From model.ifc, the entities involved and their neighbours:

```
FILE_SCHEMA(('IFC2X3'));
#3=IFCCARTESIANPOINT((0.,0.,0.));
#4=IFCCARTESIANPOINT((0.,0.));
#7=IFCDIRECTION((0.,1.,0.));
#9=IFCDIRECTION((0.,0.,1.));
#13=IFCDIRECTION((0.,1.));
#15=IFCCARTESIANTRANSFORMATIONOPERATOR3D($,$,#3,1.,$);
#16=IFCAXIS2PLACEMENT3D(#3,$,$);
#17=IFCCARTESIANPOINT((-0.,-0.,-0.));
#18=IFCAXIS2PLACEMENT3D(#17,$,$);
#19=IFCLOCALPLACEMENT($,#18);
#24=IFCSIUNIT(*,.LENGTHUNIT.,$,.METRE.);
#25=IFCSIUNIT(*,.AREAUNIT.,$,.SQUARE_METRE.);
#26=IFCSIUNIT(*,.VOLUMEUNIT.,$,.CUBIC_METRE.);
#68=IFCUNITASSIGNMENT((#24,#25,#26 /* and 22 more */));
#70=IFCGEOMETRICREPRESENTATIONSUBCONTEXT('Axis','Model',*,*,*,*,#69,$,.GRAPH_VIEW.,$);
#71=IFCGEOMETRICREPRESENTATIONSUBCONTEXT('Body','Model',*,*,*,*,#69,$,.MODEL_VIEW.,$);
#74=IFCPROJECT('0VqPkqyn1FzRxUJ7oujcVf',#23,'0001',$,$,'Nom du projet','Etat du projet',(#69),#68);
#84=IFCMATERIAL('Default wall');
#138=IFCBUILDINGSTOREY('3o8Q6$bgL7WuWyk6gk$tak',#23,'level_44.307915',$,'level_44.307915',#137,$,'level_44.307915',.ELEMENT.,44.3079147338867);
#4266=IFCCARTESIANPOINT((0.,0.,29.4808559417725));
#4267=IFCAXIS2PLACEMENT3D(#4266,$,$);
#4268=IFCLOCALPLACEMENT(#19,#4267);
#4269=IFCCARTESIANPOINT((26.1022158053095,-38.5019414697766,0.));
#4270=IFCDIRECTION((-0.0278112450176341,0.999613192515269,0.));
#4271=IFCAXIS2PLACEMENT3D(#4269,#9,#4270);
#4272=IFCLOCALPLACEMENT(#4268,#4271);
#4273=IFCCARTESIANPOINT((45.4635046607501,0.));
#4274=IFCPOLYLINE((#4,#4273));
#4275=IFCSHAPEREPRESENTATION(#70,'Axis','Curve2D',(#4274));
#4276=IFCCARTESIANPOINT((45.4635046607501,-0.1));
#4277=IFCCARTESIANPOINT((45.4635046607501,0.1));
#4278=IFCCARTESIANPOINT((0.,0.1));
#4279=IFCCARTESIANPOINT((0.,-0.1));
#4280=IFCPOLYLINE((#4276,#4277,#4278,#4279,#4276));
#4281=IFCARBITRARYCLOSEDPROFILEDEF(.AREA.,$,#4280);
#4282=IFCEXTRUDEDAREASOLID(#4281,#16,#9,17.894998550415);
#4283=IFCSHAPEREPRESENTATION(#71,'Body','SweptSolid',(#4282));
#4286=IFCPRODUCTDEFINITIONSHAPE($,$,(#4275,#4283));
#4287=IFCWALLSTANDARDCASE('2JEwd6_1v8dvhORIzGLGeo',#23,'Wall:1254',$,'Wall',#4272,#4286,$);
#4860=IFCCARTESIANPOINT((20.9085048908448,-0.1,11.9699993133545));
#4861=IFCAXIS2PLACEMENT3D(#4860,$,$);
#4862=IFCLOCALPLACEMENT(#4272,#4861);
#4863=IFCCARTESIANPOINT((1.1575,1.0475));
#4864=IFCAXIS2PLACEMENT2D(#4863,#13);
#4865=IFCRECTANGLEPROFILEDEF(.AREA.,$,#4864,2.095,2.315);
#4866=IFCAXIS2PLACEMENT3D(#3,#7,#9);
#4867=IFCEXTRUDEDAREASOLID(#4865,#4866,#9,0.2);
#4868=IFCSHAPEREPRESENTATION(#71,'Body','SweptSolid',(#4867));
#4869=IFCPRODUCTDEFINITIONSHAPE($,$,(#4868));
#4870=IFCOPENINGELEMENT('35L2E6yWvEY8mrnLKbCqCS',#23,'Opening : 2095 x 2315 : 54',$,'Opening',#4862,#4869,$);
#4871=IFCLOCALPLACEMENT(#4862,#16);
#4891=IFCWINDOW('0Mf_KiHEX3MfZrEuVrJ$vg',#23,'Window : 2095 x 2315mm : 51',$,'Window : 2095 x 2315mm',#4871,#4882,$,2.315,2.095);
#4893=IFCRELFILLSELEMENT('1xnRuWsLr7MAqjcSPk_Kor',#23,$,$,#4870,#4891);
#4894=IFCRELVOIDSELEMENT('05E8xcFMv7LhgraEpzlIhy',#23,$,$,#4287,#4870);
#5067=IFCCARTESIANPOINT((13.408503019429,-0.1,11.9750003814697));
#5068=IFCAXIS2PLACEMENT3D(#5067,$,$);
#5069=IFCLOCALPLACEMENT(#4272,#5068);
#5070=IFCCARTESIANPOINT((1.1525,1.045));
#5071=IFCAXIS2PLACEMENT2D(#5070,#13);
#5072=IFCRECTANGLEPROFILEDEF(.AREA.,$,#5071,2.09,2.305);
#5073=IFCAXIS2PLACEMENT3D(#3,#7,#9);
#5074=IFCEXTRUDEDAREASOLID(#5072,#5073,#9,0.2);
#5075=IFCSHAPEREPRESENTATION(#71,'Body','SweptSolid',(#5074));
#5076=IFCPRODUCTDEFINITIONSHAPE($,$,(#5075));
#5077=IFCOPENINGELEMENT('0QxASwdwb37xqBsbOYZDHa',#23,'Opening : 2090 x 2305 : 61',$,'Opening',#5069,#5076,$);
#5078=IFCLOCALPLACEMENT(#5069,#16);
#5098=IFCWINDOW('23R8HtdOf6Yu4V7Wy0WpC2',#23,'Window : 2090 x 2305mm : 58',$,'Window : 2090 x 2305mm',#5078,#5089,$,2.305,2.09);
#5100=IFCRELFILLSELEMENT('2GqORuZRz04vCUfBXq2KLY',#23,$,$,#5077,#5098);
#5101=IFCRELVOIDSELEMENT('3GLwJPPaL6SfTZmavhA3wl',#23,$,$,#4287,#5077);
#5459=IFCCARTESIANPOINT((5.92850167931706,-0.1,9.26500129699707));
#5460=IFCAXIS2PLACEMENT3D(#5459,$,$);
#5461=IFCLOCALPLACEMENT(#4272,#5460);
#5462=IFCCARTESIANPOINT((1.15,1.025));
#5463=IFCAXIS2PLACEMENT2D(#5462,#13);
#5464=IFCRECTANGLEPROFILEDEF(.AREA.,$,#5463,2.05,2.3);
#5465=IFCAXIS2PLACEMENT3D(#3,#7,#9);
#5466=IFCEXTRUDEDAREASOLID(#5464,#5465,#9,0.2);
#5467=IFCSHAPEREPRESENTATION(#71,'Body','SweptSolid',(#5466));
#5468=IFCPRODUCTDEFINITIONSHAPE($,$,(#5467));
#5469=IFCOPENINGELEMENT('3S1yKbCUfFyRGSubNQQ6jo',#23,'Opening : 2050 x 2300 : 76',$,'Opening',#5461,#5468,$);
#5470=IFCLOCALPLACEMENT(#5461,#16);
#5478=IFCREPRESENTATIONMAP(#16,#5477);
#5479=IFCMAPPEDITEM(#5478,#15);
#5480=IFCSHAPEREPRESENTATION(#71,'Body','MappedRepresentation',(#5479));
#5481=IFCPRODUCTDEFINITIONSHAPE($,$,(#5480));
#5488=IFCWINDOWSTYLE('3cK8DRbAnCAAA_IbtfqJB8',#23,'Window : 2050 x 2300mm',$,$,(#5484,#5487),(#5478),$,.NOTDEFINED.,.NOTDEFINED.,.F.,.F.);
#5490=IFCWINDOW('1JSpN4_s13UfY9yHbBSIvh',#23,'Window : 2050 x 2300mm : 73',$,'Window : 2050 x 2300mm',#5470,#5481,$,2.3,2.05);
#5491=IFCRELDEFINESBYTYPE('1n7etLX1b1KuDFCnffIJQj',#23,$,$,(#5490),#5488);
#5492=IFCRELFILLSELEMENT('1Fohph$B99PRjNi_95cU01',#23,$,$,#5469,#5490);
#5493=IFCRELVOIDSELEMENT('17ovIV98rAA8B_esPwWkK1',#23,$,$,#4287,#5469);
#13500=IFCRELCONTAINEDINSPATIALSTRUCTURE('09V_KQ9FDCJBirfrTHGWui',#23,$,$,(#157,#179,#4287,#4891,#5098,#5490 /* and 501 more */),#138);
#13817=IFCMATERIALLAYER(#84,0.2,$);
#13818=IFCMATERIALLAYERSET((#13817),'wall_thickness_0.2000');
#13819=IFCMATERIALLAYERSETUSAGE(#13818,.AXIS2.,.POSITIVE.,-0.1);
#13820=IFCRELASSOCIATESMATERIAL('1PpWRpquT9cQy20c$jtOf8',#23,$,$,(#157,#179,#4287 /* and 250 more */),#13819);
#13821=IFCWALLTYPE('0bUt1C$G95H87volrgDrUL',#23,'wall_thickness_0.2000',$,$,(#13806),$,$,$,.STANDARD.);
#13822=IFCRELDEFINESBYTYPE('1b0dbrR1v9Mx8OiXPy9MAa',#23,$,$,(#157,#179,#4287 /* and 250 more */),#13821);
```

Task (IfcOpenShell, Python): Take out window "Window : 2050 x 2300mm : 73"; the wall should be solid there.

```python
import ifcopenshell
import ifcopenshell.api.feature
import ifcopenshell.api.root
import ifcopenshell.geom
import ifcopenshell.util.shape

model = ifcopenshell.open("model.ifc")
settings = ifcopenshell.geom.settings()


def volume(element):
    """Net volume in cubic metres, openings subtracted."""
    shape = ifcopenshell.geom.create_shape(settings, element)
    return ifcopenshell.util.shape.get_volume(shape.geometry)


window = model.by_guid("1JSpN4_s13UfY9yHbBSIvh")
opening = window.FillsVoids[0].RelatingOpeningElement
wall = opening.VoidsElements[0].RelatingBuildingElement
before = volume(wall)

ifcopenshell.api.root.remove_product(model, product=window)
ifcopenshell.api.feature.remove_feature(model, feature=opening)

after = volume(wall)

print(f"wall volume {before:.3f} -> {after:.3f} m3")

model.write("model_edited.ifc")
```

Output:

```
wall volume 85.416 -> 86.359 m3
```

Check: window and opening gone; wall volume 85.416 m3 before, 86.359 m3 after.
